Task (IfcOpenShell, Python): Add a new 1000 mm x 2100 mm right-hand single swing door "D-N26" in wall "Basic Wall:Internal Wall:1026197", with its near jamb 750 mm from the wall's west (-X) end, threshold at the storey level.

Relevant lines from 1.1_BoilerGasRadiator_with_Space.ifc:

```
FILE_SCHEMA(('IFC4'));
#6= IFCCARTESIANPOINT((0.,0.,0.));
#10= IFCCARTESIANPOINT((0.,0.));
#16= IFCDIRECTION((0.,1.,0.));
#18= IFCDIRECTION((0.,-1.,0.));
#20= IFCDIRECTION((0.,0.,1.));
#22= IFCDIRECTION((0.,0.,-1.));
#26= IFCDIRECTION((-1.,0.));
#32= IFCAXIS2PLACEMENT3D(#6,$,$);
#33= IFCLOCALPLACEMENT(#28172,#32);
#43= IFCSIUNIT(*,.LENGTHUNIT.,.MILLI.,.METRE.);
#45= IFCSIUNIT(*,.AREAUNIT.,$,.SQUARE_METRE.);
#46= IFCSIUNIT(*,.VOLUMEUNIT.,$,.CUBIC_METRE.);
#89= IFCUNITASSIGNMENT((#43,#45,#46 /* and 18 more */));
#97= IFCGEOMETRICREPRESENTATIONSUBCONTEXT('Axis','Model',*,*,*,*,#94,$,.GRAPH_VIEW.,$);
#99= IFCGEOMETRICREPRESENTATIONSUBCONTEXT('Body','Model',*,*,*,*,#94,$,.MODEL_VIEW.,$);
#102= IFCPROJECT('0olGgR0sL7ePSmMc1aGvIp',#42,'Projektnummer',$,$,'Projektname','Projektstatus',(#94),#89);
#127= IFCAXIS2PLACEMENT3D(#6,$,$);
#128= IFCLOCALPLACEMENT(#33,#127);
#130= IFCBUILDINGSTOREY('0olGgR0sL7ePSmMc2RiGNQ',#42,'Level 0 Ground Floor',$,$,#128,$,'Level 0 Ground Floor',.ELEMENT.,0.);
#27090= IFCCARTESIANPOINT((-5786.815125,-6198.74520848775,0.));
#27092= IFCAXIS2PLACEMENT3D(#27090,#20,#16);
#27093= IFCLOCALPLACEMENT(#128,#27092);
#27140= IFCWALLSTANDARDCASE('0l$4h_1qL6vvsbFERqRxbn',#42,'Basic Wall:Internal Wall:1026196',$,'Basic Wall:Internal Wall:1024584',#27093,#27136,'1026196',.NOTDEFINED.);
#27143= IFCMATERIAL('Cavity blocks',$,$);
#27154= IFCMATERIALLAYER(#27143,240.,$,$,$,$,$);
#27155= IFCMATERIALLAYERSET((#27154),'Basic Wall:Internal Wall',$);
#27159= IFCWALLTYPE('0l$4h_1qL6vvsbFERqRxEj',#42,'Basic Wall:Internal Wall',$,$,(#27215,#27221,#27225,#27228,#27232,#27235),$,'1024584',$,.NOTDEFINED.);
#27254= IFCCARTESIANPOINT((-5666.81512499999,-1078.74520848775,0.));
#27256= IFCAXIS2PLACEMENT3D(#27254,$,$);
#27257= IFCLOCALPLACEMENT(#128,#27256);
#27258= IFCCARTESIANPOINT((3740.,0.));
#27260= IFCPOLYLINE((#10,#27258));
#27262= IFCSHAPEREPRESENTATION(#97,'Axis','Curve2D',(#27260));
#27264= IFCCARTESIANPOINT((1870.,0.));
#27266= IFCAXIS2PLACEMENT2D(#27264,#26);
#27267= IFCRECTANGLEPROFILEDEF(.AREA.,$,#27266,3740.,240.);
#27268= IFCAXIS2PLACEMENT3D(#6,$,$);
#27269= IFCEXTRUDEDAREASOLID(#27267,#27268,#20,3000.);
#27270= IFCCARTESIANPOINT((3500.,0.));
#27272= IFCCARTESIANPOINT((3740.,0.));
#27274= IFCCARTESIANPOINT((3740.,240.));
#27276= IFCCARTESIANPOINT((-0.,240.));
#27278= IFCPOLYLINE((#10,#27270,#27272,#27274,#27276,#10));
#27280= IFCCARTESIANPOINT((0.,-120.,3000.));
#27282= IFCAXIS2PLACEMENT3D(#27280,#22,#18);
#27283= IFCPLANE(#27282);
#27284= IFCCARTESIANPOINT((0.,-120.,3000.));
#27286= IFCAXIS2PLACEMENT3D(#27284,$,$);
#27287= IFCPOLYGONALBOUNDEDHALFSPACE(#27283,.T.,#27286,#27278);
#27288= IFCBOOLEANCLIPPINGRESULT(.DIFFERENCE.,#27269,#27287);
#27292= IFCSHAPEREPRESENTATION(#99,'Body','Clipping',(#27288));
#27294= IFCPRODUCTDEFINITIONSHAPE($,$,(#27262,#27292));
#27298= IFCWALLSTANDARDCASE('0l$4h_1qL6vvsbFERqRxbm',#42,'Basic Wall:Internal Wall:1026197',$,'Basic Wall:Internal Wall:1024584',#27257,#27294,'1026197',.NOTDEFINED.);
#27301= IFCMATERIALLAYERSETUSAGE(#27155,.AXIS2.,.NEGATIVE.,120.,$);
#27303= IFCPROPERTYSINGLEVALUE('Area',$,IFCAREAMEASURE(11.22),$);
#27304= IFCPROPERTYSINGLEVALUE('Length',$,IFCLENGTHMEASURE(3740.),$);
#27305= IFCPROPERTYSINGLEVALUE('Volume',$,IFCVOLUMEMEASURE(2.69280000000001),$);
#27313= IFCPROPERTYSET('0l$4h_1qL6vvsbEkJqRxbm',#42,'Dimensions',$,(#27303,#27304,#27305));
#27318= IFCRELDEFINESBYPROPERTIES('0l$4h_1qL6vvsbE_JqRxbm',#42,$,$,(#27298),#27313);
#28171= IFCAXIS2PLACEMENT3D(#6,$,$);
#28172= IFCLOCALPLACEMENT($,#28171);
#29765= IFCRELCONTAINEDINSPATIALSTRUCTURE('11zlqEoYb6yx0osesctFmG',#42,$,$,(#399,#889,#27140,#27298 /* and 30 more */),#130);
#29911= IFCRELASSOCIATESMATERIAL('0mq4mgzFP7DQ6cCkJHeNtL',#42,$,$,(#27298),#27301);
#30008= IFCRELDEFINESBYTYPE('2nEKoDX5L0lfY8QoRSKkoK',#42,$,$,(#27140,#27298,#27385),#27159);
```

```python
import numpy as np
import ifcopenshell
import ifcopenshell.api.feature
import ifcopenshell.api.geometry
import ifcopenshell.api.pset
import ifcopenshell.api.root
import ifcopenshell.api.spatial
import ifcopenshell.geom
import ifcopenshell.util.element
import ifcopenshell.util.placement
import ifcopenshell.util.representation
import ifcopenshell.util.shape
import ifcopenshell.util.unit

model = ifcopenshell.open("1.1_BoilerGasRadiator_with_Space.ifc")
unit_scale = ifcopenshell.util.unit.calculate_unit_scale(model)
area_scale = ifcopenshell.util.unit.calculate_unit_scale(model, "AREAUNIT")
volume_scale = ifcopenshell.util.unit.calculate_unit_scale(model, "VOLUMEUNIT")
settings = ifcopenshell.geom.settings()


def volume(element):
    """Net volume in cubic metres, openings subtracted."""
    shape = ifcopenshell.geom.create_shape(settings, element)
    return ifcopenshell.util.shape.get_volume(shape.geometry)


wall = model.by_guid("0l$4h_1qL6vvsbFERqRxbm")
storey = ifcopenshell.util.element.get_container(wall, ifc_class="IfcBuildingStorey")
context = ifcopenshell.util.representation.get_context(model, "Model", "Body", "MODEL_VIEW")
before = volume(wall)

width, height, from_end, sill = 1, 2.1, 0.75, 0.0  # metres

# The wall runs along its own X axis, and the end named is its -X end.
wall_shape = ifcopenshell.geom.create_shape(settings, wall)
x, y, z = ifcopenshell.util.shape.get_vertices(wall_shape.geometry).T
start = x.min() + from_end
face, thickness = float(y.min()), float(y.max() - y.min())
wall_matrix = ifcopenshell.util.placement.get_local_placement(wall.ObjectPlacement)
level = ifcopenshell.util.placement.get_local_placement(storey.ObjectPlacement)[2, 3]


def in_wall(x, y):
    """Placement at x, y metres in the wall's axes, at sill height."""
    matrix = wall_matrix.copy()
    matrix[:, 3] = wall_matrix @ np.array([x / unit_scale, y / unit_scale, 0.0, 1.0])
    matrix[2, 3] = level + sill / unit_scale
    return matrix


# Opening: a box that overshoots both wall faces by 50 mm.
opening = ifcopenshell.api.root.create_entity(model, ifc_class="IfcOpeningElement", predefined_type="OPENING")
box = ifcopenshell.api.geometry.add_wall_representation(
    model, context=context, length=width, height=height, thickness=thickness + 0.1
)
ifcopenshell.api.geometry.assign_representation(model, product=opening, representation=box)
ifcopenshell.api.geometry.edit_object_placement(model, product=opening, matrix=in_wall(start, face - 0.05), is_si=False)
ifcopenshell.api.feature.add_feature(model, feature=opening, element=wall)

door = ifcopenshell.api.root.create_entity(model, ifc_class="IfcDoor", name="D-N26", predefined_type="DOOR")
door.OverallWidth, door.OverallHeight = width / unit_scale, height / unit_scale
door.OperationType = "SINGLE_SWING_RIGHT"
body = ifcopenshell.api.geometry.add_door_representation(
    model,
    context=context,
    overall_width=door.OverallWidth,
    overall_height=door.OverallHeight,
    operation_type="SINGLE_SWING_RIGHT",
    lining_properties={"LiningDepth": thickness / unit_scale, "ThresholdDepth": thickness / unit_scale},
)
ifcopenshell.api.geometry.assign_representation(model, product=door, representation=body)
ifcopenshell.api.spatial.assign_container(model, products=[door], relating_structure=storey)
ifcopenshell.api.feature.add_filling(model, opening=opening, element=door)

# The lining spans the wall, so the door starts at the wall face.
ifcopenshell.api.geometry.edit_object_placement(model, product=door, matrix=in_wall(start, face), is_si=False)

after = volume(wall)

# Update the wall's stored quantities.
pset = model.by_id(ifcopenshell.util.element.get_pset(wall, "Dimensions", should_inherit=False)["id"])
ifcopenshell.api.pset.edit_pset(model, pset=pset, properties={
    "Area": model.create_entity("IfcAreaMeasure", after / thickness / area_scale),
    "Volume": model.create_entity("IfcVolumeMeasure", after / volume_scale),
})

print(f"wall volume {before:.3f} -> {after:.3f} m3")

model.write("1.1_BoilerGasRadiator_with_Space_rev.ifc")
```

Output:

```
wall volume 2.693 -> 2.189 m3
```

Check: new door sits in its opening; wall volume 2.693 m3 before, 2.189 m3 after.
